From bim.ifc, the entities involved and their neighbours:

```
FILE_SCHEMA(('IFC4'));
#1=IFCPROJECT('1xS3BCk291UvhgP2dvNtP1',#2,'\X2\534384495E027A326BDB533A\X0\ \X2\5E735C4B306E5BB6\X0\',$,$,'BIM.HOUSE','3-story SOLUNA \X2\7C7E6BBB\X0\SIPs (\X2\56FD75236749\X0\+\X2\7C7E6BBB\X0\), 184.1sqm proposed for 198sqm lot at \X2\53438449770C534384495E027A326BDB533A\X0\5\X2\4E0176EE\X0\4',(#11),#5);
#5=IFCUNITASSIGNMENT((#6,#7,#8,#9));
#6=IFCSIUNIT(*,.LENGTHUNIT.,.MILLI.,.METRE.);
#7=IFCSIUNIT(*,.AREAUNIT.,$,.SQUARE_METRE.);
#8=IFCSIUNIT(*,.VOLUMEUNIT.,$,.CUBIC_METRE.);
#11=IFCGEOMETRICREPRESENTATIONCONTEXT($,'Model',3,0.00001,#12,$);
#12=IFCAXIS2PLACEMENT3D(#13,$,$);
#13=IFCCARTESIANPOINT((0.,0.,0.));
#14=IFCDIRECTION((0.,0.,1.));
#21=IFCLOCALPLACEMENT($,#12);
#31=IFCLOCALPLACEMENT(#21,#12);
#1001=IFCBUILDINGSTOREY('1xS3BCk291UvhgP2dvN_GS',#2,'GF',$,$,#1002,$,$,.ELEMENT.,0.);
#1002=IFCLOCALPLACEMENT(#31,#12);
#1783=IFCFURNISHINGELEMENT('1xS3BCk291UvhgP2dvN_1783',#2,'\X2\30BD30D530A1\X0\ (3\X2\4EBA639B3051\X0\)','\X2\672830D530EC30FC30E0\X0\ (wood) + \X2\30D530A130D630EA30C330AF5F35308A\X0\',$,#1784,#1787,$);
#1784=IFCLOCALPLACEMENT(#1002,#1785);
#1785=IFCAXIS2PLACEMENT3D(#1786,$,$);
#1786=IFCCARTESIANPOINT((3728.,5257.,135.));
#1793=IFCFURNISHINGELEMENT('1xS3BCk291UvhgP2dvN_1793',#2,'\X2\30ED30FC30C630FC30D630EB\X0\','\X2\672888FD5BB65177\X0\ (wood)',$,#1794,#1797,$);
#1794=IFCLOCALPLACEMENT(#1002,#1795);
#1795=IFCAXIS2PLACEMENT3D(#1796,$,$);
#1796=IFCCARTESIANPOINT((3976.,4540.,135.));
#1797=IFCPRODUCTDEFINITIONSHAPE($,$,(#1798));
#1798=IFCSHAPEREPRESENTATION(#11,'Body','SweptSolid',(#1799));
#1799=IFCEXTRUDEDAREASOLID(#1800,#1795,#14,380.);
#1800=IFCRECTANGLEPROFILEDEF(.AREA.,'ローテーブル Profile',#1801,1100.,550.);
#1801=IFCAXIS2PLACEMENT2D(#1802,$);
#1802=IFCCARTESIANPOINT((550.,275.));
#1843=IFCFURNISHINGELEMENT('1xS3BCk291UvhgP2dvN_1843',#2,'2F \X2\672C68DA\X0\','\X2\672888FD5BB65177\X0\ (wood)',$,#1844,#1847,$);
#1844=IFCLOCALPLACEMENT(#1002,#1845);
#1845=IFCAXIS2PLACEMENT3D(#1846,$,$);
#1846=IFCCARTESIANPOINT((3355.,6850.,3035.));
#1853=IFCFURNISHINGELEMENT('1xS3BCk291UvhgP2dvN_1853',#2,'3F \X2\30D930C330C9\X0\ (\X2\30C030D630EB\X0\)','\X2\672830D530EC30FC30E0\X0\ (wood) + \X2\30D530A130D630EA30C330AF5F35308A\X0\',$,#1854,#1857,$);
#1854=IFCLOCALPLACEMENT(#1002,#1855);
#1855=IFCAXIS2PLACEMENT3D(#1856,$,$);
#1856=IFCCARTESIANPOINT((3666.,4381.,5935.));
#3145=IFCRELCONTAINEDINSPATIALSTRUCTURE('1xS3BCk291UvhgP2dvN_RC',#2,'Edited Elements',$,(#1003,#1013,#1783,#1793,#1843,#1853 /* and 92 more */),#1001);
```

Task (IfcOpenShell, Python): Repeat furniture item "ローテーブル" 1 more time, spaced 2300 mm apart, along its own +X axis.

```python
import ifcopenshell
import ifcopenshell.api.geometry
import ifcopenshell.api.root
import ifcopenshell.util.element
import ifcopenshell.util.placement
import ifcopenshell.util.unit

model = ifcopenshell.open("bim.ifc")
unit_scale = ifcopenshell.util.unit.calculate_unit_scale(model)


def reuse_history(source, copy):
    """copy_class also copies each property set's owner history, people and application; keep the originals."""
    for rel in copy.IsDefinedBy:
        if rel.is_a("IfcRelDefinesByProperties") and (history := rel.RelatingPropertyDefinition.OwnerHistory):
            rel.RelatingPropertyDefinition.OwnerHistory = source.OwnerHistory
            ifcopenshell.util.element.remove_deep2(model, history)


source = model.by_guid("1xS3BCk291UvhgP2dvN_1793")
base = ifcopenshell.util.placement.get_local_placement(source.ObjectPlacement)
step = base[:3, 0] * 2.3 / unit_scale

for i in range(1, 2):
    copy = ifcopenshell.api.root.copy_class(model, product=source)
    copy.Representation = ifcopenshell.util.element.copy_deep(
        model, source.Representation, exclude=["IfcGeometricRepresentationContext", "IfcRepresentationMap"]
    )
    reuse_history(source, copy)
    matrix = base.copy()
    matrix[:3, 3] += i * step
    print("added at", matrix[:3, 3].round(3) + 0.0)
    ifcopenshell.api.geometry.edit_object_placement(model, product=copy, matrix=matrix, is_si=False)

model.write("bim_v2.ifc")
```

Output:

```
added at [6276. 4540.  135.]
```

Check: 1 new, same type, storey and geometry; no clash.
